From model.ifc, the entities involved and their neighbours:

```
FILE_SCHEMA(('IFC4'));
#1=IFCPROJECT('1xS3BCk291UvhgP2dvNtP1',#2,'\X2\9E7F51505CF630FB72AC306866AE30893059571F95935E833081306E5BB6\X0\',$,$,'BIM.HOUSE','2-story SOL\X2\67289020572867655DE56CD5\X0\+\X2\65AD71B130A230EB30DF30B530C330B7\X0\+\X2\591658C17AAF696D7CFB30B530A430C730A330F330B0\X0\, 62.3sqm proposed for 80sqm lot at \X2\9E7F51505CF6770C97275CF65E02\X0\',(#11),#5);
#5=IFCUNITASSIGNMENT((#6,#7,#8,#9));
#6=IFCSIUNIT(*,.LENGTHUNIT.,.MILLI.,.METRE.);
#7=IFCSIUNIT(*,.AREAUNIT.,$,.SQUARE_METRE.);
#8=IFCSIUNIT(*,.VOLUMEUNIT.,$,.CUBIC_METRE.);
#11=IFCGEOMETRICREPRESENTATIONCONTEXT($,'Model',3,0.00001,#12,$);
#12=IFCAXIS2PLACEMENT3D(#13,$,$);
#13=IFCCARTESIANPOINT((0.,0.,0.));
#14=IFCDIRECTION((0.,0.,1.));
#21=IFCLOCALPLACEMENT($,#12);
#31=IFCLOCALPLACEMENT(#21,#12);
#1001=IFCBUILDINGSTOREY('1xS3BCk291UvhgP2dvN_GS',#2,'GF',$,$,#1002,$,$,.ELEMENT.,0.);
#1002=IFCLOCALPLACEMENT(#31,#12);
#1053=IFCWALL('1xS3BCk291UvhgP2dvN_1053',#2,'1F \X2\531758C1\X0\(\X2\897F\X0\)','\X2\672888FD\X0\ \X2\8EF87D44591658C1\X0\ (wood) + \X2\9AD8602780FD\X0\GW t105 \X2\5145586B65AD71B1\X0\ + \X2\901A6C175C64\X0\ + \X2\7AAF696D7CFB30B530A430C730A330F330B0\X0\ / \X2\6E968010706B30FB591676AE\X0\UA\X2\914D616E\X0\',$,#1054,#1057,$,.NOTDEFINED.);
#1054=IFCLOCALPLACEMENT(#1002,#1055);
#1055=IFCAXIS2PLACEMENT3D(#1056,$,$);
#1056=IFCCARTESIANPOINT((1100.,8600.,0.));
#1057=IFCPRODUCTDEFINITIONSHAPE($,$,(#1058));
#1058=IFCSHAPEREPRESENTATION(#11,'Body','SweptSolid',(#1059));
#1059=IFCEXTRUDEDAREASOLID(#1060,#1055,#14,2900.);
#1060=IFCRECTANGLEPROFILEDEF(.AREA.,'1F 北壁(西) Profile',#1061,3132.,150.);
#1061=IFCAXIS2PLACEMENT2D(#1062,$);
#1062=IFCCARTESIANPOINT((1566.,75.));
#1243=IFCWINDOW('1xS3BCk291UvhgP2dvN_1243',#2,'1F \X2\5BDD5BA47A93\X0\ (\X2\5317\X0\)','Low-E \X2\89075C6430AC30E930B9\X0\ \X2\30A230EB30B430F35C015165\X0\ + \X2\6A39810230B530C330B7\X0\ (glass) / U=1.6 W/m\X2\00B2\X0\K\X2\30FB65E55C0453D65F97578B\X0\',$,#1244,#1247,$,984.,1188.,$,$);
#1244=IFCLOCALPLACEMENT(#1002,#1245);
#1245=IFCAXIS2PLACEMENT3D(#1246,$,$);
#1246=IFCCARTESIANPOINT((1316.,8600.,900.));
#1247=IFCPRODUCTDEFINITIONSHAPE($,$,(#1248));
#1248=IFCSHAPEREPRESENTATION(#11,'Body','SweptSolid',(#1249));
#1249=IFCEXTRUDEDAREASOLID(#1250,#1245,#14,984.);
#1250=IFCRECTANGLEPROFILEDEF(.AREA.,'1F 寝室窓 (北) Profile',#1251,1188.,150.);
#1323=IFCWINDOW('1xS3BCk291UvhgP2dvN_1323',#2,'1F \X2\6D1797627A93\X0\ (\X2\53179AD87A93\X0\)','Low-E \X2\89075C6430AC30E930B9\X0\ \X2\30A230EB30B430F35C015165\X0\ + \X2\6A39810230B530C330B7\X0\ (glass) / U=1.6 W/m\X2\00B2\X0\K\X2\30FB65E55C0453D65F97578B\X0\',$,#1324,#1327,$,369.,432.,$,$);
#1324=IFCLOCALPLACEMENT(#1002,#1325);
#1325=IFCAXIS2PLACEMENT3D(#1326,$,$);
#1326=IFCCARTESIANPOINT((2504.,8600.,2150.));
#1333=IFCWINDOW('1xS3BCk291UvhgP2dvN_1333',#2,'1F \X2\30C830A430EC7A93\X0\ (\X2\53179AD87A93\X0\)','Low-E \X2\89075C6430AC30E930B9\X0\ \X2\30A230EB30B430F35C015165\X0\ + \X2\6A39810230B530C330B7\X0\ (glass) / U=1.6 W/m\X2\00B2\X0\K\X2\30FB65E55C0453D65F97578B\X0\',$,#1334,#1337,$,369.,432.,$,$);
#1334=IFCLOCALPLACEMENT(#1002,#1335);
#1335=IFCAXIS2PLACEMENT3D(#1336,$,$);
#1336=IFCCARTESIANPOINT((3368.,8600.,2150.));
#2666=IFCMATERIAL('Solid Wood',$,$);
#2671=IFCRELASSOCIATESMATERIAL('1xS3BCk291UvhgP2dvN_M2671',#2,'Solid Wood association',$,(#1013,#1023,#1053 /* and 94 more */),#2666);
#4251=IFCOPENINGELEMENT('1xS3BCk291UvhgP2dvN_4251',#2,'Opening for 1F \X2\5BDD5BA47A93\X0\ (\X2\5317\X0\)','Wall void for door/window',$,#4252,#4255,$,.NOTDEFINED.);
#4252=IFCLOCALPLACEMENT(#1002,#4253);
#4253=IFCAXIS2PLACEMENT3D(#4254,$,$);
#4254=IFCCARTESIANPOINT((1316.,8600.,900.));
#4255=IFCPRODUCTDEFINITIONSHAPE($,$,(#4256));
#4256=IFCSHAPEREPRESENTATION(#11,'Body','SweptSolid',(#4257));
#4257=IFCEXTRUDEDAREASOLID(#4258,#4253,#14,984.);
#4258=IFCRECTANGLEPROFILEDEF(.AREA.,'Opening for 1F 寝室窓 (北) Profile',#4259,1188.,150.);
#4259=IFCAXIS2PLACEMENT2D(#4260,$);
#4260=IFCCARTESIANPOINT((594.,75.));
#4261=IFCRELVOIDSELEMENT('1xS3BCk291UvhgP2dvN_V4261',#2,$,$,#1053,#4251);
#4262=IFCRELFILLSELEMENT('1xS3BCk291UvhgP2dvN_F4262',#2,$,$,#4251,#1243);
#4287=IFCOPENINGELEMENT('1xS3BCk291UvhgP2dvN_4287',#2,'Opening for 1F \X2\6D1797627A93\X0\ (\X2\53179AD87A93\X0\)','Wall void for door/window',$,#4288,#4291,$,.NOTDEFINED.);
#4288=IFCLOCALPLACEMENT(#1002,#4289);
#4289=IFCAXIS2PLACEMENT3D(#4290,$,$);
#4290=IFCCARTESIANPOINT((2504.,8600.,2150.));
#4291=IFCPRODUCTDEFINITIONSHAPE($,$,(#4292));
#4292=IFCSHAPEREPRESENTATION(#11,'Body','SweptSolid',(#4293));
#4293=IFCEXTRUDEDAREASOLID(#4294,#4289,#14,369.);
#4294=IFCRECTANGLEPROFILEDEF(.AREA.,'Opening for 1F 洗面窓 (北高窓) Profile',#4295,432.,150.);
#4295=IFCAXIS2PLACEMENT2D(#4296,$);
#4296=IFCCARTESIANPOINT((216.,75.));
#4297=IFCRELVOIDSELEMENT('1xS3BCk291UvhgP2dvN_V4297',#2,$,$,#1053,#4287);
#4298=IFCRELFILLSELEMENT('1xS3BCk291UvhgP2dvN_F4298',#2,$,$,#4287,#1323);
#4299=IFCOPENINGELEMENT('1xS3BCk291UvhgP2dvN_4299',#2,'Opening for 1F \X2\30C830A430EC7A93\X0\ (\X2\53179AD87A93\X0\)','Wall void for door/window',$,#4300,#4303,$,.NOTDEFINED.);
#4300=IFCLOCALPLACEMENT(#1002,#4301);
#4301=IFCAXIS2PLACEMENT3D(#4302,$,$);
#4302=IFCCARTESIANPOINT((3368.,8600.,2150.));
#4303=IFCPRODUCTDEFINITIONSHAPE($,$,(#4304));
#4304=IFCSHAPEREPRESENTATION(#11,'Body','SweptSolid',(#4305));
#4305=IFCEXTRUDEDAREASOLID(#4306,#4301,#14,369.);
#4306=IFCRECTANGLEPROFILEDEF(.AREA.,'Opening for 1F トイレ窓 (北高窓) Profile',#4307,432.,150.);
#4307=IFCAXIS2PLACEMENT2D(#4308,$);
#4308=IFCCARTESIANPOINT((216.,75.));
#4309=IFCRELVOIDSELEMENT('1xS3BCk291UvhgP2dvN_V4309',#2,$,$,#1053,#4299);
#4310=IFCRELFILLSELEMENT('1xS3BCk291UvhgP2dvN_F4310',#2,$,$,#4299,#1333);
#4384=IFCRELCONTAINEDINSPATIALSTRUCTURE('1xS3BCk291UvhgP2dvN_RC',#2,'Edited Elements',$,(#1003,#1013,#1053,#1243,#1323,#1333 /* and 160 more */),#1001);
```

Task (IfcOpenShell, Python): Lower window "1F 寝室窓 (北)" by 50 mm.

```python
import numpy as np
import ifcopenshell
import ifcopenshell.api.geometry
import ifcopenshell.util.placement
import ifcopenshell.util.unit

model = ifcopenshell.open("model.ifc")
unit_scale = ifcopenshell.util.unit.calculate_unit_scale(model)

window = model.by_guid("1xS3BCk291UvhgP2dvN_1243")
opening = window.FillsVoids[0].RelatingOpeningElement
dz = -50.0

shift = np.array([0.0, 0.0, dz])
# The window is not placed relative to its opening, so move both.
for product in (opening, window):
    matrix = ifcopenshell.util.placement.get_local_placement(product.ObjectPlacement)
    matrix[:3, 3] += shift
    ifcopenshell.api.geometry.edit_object_placement(model, product=product, matrix=matrix, is_si=False)

print(f"moved by {dz * unit_scale:+.3f} m")

model.write("model_edited.ifc")
```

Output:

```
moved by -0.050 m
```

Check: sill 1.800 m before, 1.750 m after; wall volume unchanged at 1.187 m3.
